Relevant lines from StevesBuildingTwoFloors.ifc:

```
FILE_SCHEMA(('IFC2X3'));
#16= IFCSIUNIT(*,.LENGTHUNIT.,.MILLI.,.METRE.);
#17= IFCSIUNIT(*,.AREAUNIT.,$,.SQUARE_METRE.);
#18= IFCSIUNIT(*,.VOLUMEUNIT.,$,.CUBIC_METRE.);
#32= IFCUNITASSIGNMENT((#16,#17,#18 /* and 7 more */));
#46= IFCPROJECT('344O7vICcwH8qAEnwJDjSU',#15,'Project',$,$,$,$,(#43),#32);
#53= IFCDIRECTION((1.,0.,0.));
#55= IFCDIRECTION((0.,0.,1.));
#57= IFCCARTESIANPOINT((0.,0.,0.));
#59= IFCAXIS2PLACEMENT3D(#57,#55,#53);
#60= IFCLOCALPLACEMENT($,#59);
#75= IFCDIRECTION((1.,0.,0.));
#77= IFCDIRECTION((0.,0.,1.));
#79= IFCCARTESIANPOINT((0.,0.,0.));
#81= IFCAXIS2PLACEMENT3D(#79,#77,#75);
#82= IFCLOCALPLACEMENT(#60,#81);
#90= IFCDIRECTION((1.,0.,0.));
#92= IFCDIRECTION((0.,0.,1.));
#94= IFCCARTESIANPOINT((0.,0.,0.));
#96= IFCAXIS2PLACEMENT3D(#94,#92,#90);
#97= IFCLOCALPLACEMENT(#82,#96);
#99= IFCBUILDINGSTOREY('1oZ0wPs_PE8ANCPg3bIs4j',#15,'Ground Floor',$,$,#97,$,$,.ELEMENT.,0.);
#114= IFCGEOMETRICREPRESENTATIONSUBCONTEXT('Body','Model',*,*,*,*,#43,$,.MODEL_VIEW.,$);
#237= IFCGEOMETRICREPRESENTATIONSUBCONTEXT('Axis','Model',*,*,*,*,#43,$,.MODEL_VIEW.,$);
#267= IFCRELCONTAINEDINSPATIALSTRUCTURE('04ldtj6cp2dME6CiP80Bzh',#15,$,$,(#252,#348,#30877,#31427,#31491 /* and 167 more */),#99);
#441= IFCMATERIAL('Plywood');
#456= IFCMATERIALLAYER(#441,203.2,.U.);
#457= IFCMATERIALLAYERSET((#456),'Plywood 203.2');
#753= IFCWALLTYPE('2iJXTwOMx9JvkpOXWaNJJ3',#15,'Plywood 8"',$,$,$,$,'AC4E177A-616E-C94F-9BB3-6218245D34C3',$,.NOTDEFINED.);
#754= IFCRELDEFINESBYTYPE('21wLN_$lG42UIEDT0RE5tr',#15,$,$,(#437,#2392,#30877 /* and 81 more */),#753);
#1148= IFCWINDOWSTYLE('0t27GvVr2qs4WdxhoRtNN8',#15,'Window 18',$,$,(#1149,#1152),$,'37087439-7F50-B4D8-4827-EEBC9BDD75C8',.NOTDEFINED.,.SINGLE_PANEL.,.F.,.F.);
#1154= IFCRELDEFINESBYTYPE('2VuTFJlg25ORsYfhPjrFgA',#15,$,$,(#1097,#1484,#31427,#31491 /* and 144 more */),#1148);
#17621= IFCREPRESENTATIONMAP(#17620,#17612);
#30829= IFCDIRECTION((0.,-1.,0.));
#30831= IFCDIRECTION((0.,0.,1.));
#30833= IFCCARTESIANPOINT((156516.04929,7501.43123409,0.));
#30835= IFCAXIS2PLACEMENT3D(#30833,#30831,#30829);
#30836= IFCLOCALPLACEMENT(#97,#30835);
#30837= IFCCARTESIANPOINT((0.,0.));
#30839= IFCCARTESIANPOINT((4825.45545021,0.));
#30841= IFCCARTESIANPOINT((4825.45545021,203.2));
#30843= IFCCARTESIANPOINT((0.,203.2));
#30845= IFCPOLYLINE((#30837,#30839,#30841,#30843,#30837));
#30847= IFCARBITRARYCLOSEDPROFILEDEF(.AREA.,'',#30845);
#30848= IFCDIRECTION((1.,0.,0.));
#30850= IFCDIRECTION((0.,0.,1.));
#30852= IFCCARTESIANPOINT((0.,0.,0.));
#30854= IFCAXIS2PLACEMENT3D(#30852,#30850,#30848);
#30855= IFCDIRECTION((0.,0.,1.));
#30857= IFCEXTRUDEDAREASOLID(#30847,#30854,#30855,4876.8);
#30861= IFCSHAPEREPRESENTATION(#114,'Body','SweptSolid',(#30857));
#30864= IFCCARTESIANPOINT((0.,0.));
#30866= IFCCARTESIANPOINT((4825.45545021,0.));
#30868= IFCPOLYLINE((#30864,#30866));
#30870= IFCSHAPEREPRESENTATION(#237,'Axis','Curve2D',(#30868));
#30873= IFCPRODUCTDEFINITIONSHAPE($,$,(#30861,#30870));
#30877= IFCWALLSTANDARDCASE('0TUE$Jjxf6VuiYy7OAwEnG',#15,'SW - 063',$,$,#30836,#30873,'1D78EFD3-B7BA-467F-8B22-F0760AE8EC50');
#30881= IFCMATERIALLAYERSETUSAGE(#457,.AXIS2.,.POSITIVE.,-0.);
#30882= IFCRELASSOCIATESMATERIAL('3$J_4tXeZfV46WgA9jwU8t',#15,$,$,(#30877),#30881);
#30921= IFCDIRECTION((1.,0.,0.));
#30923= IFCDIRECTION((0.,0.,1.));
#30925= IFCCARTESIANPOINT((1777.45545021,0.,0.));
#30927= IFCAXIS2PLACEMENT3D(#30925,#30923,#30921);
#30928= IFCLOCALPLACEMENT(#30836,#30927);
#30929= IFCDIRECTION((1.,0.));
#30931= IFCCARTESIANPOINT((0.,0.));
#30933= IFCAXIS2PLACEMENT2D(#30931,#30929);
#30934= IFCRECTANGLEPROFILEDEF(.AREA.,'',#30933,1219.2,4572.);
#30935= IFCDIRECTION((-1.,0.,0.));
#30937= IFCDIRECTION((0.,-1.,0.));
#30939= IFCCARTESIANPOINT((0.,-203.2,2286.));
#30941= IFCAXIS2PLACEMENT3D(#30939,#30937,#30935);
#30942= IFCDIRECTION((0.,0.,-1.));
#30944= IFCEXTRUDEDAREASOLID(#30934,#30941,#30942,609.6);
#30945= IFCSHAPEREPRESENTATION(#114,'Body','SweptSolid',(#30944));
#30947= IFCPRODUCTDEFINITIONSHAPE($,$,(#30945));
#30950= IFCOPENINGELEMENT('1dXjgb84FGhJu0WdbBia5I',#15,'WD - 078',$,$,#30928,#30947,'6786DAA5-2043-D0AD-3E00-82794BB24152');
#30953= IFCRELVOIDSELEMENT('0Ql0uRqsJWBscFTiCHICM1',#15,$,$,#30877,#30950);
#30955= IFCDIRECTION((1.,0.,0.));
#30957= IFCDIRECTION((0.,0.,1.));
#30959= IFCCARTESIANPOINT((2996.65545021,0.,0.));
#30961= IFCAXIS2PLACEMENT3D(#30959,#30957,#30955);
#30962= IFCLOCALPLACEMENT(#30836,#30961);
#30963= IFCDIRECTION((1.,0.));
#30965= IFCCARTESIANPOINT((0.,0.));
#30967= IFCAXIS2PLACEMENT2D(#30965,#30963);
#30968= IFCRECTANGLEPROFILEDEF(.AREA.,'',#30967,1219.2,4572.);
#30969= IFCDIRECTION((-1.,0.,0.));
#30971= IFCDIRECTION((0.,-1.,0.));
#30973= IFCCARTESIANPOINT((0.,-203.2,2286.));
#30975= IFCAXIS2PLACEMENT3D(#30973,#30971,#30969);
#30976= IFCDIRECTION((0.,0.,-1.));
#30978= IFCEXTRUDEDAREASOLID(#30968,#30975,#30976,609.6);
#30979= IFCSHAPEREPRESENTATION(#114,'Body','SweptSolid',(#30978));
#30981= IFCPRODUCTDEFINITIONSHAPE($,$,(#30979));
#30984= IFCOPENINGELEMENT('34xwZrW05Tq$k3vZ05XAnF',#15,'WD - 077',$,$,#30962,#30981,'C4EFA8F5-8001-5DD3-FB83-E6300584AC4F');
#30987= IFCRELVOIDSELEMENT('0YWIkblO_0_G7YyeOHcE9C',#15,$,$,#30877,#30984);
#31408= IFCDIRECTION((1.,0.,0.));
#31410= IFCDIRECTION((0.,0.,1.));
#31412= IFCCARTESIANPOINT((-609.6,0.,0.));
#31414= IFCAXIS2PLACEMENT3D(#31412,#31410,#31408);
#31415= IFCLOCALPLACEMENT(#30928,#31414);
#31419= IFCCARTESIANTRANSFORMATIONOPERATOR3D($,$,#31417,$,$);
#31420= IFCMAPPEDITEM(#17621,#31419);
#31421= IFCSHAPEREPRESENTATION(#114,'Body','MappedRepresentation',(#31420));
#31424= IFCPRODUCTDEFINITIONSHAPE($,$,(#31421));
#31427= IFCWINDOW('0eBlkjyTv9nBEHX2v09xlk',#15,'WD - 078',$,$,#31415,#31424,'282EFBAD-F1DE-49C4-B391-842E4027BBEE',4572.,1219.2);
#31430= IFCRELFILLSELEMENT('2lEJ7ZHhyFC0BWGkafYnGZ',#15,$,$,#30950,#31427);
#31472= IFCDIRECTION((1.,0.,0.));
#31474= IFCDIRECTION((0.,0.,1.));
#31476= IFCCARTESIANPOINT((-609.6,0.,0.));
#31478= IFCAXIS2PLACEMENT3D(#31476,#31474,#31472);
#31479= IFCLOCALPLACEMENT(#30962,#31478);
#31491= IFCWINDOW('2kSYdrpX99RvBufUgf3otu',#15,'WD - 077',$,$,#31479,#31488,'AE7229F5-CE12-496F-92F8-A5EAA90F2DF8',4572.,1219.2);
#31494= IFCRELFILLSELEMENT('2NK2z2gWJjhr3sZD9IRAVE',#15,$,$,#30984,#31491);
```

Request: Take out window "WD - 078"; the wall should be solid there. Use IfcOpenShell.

```python
import ifcopenshell
import ifcopenshell.api.feature
import ifcopenshell.api.root
import ifcopenshell.geom
import ifcopenshell.util.shape

model = ifcopenshell.open("StevesBuildingTwoFloors.ifc")
settings = ifcopenshell.geom.settings()


def volume(element):
    """Net volume in cubic metres, openings subtracted."""
    shape = ifcopenshell.geom.create_shape(settings, element)
    return ifcopenshell.util.shape.get_volume(shape.geometry)


window = model.by_guid("0eBlkjyTv9nBEHX2v09xlk")
opening = window.FillsVoids[0].RelatingOpeningElement
wall = opening.VoidsElements[0].RelatingBuildingElement
before = volume(wall)

ifcopenshell.api.root.remove_product(model, product=window)
ifcopenshell.api.feature.remove_feature(model, feature=opening)

after = volume(wall)

print(f"wall volume {before:.3f} -> {after:.3f} m3")

model.write("StevesBuildingTwoFloors_edited.ifc")
```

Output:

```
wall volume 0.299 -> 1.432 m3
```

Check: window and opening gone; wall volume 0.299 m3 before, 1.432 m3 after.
